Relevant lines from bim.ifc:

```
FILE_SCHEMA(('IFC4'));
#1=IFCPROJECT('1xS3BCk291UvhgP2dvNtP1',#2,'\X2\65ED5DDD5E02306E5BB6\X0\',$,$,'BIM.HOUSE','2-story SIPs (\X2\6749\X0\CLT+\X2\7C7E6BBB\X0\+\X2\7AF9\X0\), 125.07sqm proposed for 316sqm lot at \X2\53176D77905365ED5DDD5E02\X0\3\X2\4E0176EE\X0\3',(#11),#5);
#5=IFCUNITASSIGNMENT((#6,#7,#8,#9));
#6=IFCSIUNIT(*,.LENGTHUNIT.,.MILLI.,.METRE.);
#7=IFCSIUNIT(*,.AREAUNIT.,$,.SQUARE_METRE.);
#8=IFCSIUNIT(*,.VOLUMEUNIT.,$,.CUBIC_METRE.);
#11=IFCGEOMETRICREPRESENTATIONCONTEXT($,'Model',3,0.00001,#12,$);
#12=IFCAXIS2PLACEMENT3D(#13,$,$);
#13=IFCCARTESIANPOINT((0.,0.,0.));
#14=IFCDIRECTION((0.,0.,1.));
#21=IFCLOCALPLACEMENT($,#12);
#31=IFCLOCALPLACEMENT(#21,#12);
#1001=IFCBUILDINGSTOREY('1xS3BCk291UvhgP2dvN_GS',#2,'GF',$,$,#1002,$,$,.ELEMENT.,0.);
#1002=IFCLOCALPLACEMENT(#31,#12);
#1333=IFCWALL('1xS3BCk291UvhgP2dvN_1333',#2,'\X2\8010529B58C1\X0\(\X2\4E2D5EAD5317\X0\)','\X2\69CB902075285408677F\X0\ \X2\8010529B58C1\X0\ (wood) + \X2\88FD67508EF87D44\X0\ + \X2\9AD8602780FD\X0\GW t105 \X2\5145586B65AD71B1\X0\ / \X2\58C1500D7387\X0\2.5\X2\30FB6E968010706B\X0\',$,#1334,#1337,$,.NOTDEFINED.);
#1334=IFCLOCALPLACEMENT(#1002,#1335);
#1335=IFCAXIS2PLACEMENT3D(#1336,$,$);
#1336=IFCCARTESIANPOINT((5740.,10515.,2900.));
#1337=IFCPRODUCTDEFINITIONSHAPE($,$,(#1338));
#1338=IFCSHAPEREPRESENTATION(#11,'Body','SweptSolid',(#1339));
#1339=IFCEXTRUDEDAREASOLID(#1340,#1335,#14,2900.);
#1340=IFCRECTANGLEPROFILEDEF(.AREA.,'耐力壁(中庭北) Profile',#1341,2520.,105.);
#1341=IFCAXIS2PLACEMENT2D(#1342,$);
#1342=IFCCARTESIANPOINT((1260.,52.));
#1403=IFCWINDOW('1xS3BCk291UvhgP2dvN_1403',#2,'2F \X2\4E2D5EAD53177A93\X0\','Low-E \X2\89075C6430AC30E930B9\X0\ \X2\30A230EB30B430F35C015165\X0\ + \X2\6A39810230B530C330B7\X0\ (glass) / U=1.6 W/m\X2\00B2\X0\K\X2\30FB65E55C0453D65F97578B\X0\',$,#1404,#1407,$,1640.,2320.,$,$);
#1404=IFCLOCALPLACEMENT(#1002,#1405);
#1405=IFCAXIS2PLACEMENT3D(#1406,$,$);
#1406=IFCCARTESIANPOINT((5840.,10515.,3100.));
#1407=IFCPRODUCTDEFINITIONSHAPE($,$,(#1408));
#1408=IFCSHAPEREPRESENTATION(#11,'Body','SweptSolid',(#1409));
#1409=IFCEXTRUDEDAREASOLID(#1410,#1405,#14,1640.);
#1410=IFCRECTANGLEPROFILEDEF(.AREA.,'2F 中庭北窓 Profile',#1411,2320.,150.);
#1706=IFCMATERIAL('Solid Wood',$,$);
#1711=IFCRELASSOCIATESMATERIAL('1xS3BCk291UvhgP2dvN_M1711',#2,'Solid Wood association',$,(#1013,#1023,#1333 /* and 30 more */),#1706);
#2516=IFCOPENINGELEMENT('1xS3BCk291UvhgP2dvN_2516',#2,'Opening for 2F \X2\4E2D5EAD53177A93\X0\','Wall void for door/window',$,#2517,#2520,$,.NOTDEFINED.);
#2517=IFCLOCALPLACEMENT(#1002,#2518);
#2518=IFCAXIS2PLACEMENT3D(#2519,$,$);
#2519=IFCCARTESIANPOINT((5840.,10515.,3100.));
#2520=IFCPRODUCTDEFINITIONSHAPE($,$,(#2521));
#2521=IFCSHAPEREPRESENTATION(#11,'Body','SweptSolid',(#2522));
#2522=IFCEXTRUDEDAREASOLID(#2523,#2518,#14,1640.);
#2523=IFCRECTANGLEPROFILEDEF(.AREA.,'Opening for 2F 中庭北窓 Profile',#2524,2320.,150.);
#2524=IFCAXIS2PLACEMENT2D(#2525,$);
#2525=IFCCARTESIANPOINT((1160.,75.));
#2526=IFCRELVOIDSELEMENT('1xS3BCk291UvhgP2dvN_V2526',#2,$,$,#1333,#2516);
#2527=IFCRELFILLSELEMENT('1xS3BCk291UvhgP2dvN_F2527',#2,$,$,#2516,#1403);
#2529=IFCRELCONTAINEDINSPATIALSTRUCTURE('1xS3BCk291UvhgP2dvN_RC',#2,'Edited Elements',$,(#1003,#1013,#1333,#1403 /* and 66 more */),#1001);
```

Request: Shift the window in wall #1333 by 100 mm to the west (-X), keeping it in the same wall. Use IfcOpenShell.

```python
import ifcopenshell
import ifcopenshell.api.geometry
import ifcopenshell.util.placement
import ifcopenshell.util.unit

model = ifcopenshell.open("bim.ifc")
unit_scale = ifcopenshell.util.unit.calculate_unit_scale(model)

window = model.by_id(1403)
opening = window.FillsVoids[0].RelatingOpeningElement
wall = opening.VoidsElements[0].RelatingBuildingElement

wall_matrix = ifcopenshell.util.placement.get_local_placement(wall.ObjectPlacement)
shift = wall_matrix[:3, 0] * -0.1 / unit_scale
before = ifcopenshell.util.placement.get_local_placement(window.ObjectPlacement)[:3, 3].copy()

# The window is not placed relative to its opening, so move both.
for product in (opening, window):
    matrix = ifcopenshell.util.placement.get_local_placement(product.ObjectPlacement)
    matrix[:3, 3] += shift
    ifcopenshell.api.geometry.edit_object_placement(model, product=product, matrix=matrix, is_si=False)

after = ifcopenshell.util.placement.get_local_placement(window.ObjectPlacement)[:3, 3]
print("window moved by", (after - before).round(3) + 0.0)

model.write("bim_v2.ifc")
```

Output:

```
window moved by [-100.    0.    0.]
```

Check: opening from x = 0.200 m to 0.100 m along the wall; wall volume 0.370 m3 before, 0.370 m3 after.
